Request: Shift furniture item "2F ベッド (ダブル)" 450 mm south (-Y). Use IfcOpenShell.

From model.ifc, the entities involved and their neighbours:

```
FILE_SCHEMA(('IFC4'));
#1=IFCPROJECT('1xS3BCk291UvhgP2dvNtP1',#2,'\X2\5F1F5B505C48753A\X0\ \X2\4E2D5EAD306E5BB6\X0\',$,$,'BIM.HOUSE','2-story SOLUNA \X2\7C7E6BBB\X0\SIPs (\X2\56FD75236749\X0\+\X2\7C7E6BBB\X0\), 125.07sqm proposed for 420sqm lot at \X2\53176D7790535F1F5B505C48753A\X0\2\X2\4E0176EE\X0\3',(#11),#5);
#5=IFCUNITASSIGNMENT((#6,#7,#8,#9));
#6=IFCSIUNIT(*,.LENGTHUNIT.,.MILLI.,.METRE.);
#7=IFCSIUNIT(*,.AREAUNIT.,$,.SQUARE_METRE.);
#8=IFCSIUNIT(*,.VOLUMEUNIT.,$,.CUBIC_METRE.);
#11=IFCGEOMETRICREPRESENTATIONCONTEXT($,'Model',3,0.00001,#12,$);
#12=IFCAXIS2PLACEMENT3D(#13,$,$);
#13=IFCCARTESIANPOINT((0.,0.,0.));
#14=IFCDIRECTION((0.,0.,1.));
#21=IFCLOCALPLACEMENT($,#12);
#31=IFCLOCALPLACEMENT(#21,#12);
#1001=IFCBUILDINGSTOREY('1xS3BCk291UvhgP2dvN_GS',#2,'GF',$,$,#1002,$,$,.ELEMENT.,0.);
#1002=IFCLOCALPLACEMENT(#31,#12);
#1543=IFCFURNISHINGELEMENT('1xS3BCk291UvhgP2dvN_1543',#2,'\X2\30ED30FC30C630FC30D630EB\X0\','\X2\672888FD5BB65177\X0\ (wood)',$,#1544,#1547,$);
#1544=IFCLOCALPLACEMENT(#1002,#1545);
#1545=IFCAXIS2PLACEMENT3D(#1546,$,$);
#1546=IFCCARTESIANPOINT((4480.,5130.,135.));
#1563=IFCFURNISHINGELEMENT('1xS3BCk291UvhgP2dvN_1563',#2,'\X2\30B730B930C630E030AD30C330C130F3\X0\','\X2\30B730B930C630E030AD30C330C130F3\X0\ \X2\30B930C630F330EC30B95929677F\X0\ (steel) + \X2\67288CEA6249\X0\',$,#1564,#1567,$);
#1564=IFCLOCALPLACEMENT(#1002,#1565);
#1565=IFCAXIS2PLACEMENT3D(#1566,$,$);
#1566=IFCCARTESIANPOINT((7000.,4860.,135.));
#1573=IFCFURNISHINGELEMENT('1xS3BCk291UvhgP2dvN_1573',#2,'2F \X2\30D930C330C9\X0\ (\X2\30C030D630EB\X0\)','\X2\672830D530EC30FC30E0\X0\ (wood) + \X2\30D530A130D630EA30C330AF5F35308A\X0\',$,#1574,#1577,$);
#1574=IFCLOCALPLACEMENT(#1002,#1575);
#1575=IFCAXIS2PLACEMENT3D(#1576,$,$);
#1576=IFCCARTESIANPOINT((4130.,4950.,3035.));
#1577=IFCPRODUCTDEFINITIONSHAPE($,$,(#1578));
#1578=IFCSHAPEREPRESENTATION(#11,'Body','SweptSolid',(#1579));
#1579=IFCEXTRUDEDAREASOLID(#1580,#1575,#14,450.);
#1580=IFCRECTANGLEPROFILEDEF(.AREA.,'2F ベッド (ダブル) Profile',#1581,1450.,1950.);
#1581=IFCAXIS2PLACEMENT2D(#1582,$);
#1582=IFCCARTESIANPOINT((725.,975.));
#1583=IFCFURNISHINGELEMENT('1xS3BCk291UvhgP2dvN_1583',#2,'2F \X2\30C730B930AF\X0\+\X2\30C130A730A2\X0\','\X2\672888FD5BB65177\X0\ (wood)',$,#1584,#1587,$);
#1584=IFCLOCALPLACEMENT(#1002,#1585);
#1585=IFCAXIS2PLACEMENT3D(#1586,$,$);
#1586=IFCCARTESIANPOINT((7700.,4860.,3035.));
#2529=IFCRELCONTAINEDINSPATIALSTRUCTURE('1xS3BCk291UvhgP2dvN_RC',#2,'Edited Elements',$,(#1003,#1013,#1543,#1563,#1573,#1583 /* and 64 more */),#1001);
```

```python
import ifcopenshell
import ifcopenshell.api.geometry
import ifcopenshell.util.placement

model = ifcopenshell.open("model.ifc")

item = model.by_guid("1xS3BCk291UvhgP2dvN_1573")
matrix = ifcopenshell.util.placement.get_local_placement(item.ObjectPlacement)
matrix[1, 3] -= 450.0
ifcopenshell.api.geometry.edit_object_placement(model, product=item, matrix=matrix, is_si=False)

print(ifcopenshell.util.placement.get_local_placement(item.ObjectPlacement).round(3) + 0.0)

model.write("model-out.ifc")
```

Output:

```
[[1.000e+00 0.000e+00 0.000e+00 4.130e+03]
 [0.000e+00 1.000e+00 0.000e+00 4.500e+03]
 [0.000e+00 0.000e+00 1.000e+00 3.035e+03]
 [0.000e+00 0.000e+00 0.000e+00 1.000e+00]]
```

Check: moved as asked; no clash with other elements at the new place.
